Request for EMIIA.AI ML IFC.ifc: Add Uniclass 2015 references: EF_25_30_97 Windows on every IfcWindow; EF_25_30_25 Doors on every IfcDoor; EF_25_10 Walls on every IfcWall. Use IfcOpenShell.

First a look at what the model holds.

```python
import ifcopenshell

model = ifcopenshell.open("EMIIA.AI ML IFC.ifc")
print(model.schema)
print("classifications:", [c.Name for c in model.by_type("IfcClassification")])
for ifc_class in ("IfcDoor", "IfcRoof", "IfcStair", "IfcWall", "IfcWindow"):
    print(ifc_class, len(model.by_type(ifc_class)))
```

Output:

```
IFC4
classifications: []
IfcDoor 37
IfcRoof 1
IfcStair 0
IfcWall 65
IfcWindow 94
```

```python
import ifcopenshell
import ifcopenshell.api.classification

model = ifcopenshell.open("EMIIA.AI ML IFC.ifc")

system = ifcopenshell.api.classification.add_classification(model, classification="Uniclass 2015")

codes = {
    "IfcWindow": ("EF_25_30_97", "Windows"),
    "IfcDoor": ("EF_25_30_25", "Doors"),
    "IfcWall": ("EF_25_10", "Walls"),
}
for ifc_class, (code, name) in codes.items():
    products = model.by_type(ifc_class)
    ifcopenshell.api.classification.add_reference(
        model, products=products, classification=system, identification=code, name=name
    )
    print(code, len(products))

model.write("EMIIA.AI ML IFC-out.ifc")
```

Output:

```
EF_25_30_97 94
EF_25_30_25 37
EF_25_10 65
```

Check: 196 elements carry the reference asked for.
